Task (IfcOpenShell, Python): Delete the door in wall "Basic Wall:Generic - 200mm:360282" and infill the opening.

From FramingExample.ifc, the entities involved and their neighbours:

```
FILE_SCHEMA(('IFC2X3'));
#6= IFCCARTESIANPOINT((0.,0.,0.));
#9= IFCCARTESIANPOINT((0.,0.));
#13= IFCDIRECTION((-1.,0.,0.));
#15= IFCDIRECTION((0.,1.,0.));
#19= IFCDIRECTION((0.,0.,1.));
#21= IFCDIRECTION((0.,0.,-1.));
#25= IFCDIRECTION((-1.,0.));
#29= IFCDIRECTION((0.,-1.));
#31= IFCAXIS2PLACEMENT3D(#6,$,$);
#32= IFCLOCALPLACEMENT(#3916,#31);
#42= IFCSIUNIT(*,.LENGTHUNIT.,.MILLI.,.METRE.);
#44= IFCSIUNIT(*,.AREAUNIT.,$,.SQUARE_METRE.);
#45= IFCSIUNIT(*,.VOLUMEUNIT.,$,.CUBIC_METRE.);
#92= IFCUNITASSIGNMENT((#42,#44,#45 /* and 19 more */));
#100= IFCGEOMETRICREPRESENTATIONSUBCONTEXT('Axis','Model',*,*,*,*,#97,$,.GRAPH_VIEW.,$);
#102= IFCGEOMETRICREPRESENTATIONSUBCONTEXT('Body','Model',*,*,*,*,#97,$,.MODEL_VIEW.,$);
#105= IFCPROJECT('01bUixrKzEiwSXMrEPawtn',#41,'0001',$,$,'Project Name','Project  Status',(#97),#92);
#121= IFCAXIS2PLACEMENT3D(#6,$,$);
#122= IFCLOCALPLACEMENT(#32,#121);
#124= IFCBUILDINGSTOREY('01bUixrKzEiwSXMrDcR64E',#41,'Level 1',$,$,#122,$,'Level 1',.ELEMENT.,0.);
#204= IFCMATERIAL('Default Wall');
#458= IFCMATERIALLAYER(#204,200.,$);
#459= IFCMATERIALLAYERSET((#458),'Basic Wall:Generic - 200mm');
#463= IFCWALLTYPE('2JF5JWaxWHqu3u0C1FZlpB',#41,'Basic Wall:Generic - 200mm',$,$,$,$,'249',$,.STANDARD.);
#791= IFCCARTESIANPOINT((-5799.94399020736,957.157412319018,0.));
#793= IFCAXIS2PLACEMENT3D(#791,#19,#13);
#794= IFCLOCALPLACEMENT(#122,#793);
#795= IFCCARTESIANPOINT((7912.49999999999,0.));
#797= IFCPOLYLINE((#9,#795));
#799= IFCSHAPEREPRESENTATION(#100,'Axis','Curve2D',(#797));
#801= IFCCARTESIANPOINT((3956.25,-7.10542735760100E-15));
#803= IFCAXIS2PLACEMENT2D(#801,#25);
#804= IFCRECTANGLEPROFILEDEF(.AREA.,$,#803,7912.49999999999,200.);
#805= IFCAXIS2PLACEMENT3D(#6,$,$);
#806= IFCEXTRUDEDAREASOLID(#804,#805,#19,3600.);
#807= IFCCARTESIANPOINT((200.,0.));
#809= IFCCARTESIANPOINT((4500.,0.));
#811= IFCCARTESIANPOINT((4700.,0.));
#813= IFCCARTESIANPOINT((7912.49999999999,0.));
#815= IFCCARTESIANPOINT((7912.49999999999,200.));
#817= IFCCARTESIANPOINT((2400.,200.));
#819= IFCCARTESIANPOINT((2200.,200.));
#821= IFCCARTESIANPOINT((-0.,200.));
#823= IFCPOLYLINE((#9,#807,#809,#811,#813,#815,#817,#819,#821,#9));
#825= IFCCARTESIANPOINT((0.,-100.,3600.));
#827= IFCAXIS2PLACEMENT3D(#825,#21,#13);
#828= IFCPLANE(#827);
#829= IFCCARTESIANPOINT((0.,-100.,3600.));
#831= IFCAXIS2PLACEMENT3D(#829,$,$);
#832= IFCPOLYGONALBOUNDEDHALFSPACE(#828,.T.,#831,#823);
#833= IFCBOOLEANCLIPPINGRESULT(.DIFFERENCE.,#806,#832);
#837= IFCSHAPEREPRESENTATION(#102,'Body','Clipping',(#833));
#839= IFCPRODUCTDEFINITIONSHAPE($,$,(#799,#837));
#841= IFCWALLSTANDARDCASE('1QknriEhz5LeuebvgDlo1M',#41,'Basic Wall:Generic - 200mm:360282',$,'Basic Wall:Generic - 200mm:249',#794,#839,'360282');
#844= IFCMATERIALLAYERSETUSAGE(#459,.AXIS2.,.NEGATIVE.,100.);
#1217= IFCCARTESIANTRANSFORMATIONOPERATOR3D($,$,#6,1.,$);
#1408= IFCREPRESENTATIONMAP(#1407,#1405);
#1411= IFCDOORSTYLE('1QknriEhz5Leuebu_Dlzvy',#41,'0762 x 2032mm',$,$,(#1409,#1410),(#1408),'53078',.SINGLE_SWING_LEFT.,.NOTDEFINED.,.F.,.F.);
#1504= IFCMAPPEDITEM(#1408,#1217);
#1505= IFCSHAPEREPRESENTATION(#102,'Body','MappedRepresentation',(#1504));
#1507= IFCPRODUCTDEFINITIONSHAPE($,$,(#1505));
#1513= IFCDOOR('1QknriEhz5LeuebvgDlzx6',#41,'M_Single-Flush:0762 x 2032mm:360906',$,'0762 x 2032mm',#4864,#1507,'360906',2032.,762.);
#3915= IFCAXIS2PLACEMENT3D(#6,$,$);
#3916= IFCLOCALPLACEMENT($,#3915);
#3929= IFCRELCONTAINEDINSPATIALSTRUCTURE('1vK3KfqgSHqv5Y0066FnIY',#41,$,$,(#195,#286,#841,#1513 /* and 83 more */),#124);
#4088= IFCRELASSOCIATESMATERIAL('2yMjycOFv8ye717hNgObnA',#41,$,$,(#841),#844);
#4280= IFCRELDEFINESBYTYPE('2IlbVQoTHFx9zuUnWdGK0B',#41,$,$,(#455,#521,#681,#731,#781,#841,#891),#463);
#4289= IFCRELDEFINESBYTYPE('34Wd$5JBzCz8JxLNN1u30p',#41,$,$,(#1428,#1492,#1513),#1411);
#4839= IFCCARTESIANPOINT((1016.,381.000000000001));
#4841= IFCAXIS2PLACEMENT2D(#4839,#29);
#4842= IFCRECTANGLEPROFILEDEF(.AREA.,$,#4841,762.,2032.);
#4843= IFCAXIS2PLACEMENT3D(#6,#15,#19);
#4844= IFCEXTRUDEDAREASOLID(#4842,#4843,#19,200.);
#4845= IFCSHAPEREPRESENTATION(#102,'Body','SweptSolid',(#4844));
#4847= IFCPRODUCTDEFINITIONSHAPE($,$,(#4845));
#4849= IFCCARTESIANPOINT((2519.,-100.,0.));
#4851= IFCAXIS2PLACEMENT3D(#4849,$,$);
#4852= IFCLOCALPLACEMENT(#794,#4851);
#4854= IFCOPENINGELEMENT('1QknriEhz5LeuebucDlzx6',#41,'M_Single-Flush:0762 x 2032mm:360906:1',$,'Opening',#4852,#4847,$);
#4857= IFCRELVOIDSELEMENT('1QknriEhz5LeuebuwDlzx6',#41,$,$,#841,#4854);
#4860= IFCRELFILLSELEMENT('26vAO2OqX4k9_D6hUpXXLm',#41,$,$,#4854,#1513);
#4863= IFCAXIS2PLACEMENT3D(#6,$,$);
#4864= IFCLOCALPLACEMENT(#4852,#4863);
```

```python
import ifcopenshell
import ifcopenshell.api.feature
import ifcopenshell.api.root
import ifcopenshell.geom
import ifcopenshell.util.shape

model = ifcopenshell.open("FramingExample.ifc")
settings = ifcopenshell.geom.settings()


def volume(element):
    """Net volume in cubic metres, openings subtracted."""
    shape = ifcopenshell.geom.create_shape(settings, element)
    return ifcopenshell.util.shape.get_volume(shape.geometry)


door = model.by_guid("1QknriEhz5LeuebvgDlzx6")
opening = door.FillsVoids[0].RelatingOpeningElement
wall = opening.VoidsElements[0].RelatingBuildingElement
before = volume(wall)

ifcopenshell.api.root.remove_product(model, product=door)
ifcopenshell.api.feature.remove_feature(model, feature=opening)

after = volume(wall)

print(f"wall volume {before:.3f} -> {after:.3f} m3")

model.write("FramingExample_edited.ifc")
```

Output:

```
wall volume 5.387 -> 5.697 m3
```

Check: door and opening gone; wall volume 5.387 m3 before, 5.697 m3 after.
